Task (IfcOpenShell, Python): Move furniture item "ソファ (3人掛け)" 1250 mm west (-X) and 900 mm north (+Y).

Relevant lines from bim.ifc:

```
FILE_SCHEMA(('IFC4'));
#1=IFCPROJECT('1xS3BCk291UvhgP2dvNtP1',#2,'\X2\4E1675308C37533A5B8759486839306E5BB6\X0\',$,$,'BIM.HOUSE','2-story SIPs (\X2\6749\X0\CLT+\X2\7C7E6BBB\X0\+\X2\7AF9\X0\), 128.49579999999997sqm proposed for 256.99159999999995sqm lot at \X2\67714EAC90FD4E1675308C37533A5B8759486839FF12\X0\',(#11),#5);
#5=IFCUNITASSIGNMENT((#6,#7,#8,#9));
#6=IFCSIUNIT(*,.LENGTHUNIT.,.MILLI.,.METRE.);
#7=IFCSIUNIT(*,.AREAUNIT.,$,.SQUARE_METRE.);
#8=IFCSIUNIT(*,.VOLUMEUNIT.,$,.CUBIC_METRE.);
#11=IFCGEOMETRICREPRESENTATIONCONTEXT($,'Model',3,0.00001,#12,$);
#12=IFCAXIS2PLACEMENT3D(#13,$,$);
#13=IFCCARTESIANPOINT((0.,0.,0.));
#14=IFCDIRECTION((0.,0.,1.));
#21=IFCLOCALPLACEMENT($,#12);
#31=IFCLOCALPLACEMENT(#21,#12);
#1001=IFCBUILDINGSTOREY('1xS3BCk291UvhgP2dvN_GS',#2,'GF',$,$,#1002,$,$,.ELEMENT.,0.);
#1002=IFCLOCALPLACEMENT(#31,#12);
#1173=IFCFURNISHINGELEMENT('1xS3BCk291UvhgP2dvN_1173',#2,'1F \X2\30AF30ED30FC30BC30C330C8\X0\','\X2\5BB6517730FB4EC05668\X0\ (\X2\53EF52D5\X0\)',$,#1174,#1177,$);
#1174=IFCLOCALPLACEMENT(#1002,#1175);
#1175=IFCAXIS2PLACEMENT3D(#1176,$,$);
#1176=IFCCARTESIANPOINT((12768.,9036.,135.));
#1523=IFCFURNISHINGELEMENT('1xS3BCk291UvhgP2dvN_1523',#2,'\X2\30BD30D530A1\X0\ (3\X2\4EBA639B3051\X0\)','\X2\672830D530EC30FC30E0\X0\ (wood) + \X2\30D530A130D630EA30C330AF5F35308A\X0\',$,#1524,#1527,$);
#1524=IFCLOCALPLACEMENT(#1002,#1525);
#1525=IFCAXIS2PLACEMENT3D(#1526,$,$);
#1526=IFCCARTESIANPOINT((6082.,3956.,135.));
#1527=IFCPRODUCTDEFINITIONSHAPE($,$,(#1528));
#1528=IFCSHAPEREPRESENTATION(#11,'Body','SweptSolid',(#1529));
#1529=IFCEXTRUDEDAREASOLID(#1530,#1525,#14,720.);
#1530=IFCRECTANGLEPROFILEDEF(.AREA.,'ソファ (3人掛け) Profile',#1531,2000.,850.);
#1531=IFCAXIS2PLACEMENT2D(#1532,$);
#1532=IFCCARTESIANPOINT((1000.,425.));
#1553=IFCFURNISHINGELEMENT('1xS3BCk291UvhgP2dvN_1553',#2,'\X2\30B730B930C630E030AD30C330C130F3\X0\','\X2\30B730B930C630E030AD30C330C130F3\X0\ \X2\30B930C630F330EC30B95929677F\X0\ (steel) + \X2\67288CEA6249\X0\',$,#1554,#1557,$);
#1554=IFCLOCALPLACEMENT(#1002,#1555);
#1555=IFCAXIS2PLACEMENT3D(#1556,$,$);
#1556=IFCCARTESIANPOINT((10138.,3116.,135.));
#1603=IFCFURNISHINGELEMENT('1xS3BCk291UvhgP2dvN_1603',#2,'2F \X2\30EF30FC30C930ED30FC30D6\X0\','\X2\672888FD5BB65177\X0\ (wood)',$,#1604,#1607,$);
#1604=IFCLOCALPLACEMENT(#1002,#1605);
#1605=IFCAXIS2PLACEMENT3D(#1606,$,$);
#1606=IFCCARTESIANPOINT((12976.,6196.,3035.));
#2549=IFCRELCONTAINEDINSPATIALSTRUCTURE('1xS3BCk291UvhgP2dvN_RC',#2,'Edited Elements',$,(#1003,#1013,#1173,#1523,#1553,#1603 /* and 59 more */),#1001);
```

```python
import ifcopenshell
import ifcopenshell.api.geometry
import ifcopenshell.util.placement
import ifcopenshell.util.unit

model = ifcopenshell.open("bim.ifc")
unit_scale = ifcopenshell.util.unit.calculate_unit_scale(model)

item = model.by_guid("1xS3BCk291UvhgP2dvN_1523")
matrix = ifcopenshell.util.placement.get_local_placement(item.ObjectPlacement)
matrix[0, 3] -= 1.25 / unit_scale
matrix[1, 3] += 0.9 / unit_scale
ifcopenshell.api.geometry.edit_object_placement(model, product=item, matrix=matrix, is_si=False)

print(ifcopenshell.util.placement.get_local_placement(item.ObjectPlacement).round(3) + 0.0)

model.write("bim_v2.ifc")
```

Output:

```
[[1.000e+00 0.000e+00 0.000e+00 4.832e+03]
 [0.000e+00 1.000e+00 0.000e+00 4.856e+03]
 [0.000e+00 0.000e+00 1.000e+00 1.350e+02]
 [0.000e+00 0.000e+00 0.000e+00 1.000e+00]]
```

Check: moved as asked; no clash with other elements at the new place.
